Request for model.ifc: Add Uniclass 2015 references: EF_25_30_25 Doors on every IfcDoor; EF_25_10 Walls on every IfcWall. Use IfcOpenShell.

First a look at what the model holds.

```python
import ifcopenshell

model = ifcopenshell.open("model.ifc")
print(model.schema)
print("classifications:", [c.Name for c in model.by_type("IfcClassification")])
for ifc_class in ("IfcDoor", "IfcRoof", "IfcStair", "IfcWall", "IfcWindow"):
    print(ifc_class, len(model.by_type(ifc_class)))
```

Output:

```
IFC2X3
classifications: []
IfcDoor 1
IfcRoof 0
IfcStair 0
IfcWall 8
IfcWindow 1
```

```python
import ifcopenshell
import ifcopenshell.api.classification

model = ifcopenshell.open("model.ifc")

# IFC2X3 requires Source and Edition and has no link from the project to the system.
system = model.create_entity("IfcClassification", Source="NBS", Edition="2015", Name="Uniclass 2015")

codes = {
    "IfcDoor": ("EF_25_30_25", "Doors"),
    "IfcWall": ("EF_25_10", "Walls"),
}
for ifc_class, (code, name) in codes.items():
    products = model.by_type(ifc_class)
    ifcopenshell.api.classification.add_reference(
        model, products=products, classification=system, identification=code, name=name
    )
    print(code, len(products))

model.write("model-out.ifc")
```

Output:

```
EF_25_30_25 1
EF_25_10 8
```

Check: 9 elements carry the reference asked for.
